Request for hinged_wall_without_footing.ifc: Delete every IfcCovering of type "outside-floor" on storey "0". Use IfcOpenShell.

First a look at what the model holds.

```python
import ifcopenshell
import ifcopenshell.util.element

model = ifcopenshell.open("hinged_wall_without_footing.ifc")
print(model.schema)
storey = next(s for s in model.by_type("IfcBuildingStorey") if s.Name == "0")
coverings = [e for e in ifcopenshell.util.element.get_decomposition(storey) if e.is_a("IfcCovering")]
seen = {}
for e in coverings:
    element_type = ifcopenshell.util.element.get_type(e)
    name = element_type.Name if element_type not in (None, e) else None
    seen[name] = seen.get(name, 0) + 1
for name, count in sorted(seen.items(), key=str):
    print(count, "x", name)
```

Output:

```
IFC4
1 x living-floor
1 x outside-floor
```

```python
import ifcopenshell
import ifcopenshell.api.root
import ifcopenshell.util.element

model = ifcopenshell.open("hinged_wall_without_footing.ifc")

storey = next(s for s in model.by_type("IfcBuildingStorey") if s.Name == "0")
coverings = [e for e in ifcopenshell.util.element.get_decomposition(storey) if e.is_a("IfcCovering")]
targets = [e for e in coverings if (t := ifcopenshell.util.element.get_type(e)) not in (None, e) and t.Name == "outside-floor"]

for e in targets:
    ifcopenshell.api.root.remove_product(model, product=e)
print(len(targets), "removed")

model.write("hinged_wall_without_footing_rev.ifc")
```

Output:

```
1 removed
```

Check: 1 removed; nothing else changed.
